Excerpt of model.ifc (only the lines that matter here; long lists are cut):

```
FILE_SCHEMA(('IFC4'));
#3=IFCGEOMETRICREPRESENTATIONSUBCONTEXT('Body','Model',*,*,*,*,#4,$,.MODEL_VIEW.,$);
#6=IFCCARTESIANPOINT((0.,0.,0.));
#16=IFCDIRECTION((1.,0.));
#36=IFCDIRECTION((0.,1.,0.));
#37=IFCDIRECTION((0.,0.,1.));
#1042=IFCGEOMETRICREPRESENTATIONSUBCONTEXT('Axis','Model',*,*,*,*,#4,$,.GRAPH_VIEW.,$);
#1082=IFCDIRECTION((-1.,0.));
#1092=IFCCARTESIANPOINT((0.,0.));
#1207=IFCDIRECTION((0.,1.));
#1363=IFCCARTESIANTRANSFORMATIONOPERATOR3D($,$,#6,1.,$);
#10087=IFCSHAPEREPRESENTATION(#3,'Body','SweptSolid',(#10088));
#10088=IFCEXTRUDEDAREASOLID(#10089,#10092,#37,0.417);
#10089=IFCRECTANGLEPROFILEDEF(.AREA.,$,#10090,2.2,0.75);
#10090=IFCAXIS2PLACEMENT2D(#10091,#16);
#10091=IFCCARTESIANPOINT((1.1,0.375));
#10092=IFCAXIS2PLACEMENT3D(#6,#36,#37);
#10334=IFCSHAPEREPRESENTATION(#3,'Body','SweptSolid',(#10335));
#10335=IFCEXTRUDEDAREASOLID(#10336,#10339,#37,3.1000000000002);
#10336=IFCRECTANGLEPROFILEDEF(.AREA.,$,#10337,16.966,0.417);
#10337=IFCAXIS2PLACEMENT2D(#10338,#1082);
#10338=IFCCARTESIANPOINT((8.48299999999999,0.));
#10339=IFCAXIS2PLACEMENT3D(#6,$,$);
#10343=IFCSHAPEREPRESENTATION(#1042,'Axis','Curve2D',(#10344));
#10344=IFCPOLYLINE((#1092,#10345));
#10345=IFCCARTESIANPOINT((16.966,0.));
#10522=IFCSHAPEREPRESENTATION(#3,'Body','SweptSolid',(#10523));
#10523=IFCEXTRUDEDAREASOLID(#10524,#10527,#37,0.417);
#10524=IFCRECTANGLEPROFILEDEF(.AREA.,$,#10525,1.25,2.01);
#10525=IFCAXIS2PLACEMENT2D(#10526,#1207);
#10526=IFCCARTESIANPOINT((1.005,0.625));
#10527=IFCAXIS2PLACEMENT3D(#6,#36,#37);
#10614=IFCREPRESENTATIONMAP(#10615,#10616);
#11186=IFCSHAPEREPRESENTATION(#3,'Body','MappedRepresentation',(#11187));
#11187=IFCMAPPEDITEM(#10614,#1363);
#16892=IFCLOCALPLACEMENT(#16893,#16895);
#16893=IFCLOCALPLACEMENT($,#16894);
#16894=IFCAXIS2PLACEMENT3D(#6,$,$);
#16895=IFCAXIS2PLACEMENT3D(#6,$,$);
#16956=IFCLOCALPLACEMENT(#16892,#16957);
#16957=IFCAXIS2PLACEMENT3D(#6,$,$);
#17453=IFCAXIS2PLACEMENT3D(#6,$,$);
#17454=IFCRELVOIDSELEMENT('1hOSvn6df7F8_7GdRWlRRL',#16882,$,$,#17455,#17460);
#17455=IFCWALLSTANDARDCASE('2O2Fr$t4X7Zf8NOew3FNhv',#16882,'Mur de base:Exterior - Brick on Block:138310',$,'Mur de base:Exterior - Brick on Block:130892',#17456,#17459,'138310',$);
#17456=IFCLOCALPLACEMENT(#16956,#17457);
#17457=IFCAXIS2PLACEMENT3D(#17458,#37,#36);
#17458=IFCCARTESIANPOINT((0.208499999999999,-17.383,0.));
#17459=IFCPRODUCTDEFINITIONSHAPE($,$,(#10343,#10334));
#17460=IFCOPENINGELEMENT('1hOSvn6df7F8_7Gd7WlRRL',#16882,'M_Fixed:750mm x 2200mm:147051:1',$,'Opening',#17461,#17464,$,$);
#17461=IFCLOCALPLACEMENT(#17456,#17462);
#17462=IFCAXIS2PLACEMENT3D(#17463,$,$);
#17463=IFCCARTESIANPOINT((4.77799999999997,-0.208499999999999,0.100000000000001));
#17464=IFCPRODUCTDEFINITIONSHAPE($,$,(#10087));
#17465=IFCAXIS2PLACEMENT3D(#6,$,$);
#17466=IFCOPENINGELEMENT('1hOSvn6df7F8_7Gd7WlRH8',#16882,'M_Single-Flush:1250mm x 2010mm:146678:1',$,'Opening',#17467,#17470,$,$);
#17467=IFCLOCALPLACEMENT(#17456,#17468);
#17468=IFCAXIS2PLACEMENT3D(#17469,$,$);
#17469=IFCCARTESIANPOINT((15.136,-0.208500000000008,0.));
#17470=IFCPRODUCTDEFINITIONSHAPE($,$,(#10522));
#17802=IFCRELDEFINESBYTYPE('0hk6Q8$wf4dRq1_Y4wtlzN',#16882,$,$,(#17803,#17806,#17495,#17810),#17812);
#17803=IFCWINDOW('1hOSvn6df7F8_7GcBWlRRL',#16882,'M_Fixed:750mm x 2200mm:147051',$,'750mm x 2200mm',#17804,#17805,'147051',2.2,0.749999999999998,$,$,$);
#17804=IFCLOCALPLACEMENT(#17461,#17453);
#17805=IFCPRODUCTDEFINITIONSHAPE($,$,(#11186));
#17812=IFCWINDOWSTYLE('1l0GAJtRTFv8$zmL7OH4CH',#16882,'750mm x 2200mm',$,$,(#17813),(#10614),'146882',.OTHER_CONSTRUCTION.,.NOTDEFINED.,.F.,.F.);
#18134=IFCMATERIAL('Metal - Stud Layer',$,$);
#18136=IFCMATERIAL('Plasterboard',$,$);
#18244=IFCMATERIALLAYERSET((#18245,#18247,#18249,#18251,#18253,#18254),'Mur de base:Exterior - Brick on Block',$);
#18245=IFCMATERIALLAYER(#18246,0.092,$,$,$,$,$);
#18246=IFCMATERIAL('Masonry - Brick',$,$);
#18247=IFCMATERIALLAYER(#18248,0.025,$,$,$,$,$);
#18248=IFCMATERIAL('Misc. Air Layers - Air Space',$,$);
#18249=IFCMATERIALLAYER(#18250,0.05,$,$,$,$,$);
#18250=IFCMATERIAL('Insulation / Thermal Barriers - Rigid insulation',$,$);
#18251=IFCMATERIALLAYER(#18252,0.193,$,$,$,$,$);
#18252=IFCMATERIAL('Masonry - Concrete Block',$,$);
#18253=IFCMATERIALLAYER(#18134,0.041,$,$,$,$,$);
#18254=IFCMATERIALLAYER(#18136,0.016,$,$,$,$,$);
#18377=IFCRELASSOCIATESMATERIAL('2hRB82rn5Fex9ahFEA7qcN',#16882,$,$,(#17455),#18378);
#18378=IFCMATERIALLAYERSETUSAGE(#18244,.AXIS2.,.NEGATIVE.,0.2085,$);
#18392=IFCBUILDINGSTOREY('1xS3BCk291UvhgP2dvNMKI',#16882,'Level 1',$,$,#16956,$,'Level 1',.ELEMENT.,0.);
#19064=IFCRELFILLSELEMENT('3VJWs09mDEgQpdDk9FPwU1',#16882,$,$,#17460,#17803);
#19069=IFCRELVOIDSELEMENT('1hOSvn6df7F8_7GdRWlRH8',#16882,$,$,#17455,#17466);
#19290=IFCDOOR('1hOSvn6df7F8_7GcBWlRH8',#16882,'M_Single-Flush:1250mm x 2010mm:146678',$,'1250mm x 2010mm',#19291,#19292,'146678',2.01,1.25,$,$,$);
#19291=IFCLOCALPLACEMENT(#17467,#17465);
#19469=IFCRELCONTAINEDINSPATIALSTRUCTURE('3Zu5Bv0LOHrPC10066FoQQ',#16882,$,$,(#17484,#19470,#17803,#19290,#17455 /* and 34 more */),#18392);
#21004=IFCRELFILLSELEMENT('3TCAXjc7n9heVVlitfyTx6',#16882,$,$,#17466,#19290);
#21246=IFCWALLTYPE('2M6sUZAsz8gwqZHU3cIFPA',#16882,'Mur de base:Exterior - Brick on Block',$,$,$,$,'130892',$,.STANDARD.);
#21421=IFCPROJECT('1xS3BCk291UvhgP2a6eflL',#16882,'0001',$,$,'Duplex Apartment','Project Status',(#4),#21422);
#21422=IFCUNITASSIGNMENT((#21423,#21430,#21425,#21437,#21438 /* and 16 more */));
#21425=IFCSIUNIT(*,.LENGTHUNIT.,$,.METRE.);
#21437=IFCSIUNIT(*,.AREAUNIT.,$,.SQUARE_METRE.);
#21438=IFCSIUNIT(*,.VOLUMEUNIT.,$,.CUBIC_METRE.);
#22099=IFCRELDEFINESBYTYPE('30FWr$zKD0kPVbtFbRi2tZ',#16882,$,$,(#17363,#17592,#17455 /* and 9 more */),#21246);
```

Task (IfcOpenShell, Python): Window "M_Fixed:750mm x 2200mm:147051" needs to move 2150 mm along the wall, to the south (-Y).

```python
import ifcopenshell
import ifcopenshell.api.geometry
import ifcopenshell.util.placement

model = ifcopenshell.open("model.ifc")

window = model.by_id(17803)
opening = window.FillsVoids[0].RelatingOpeningElement
wall = opening.VoidsElements[0].RelatingBuildingElement

wall_matrix = ifcopenshell.util.placement.get_local_placement(wall.ObjectPlacement)
shift = wall_matrix[:3, 0] * -2.15
before = ifcopenshell.util.placement.get_local_placement(window.ObjectPlacement)[:3, 3].copy()

# The window is placed relative to its opening, so it follows when the opening moves.
matrix = ifcopenshell.util.placement.get_local_placement(opening.ObjectPlacement)
matrix[:3, 3] += shift
ifcopenshell.api.geometry.edit_object_placement(
    model, product=opening, matrix=matrix, is_si=False, should_transform_children=True
)

after = ifcopenshell.util.placement.get_local_placement(window.ObjectPlacement)[:3, 3]
print("window moved by", (after - before).round(3) + 0.0)

model.write("model-out.ifc")
```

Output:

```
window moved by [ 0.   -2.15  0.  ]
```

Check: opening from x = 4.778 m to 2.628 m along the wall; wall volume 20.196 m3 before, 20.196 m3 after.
